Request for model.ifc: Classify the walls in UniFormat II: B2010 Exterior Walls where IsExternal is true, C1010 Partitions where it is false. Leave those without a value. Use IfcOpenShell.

First a look at what the model holds.

```python
import ifcopenshell
import ifcopenshell.util.element

model = ifcopenshell.open("model.ifc")
print(model.schema)
print("classifications:", [c.Name for c in model.by_type("IfcClassification")])
values = [ifcopenshell.util.element.get_pset(e, "Pset_WallCommon", "IsExternal") for e in model.by_type("IfcWall")]
for value in (True, False, None):
    print("IsExternal", value, values.count(value))
```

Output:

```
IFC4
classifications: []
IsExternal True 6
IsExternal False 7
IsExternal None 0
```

```python
import ifcopenshell
import ifcopenshell.api.classification
import ifcopenshell.util.element

model = ifcopenshell.open("model.ifc")

system = ifcopenshell.api.classification.add_classification(model, classification="UniFormat II")

walls = model.by_type("IfcWall")
external = {e: ifcopenshell.util.element.get_pset(e, "Pset_WallCommon", "IsExternal") for e in walls}
for flag, code, name in ((True, "B2010", "Exterior Walls"), (False, "C1010", "Partitions")):
    products = [e for e in walls if external[e] is flag]
    ifcopenshell.api.classification.add_reference(
        model, products=products, classification=system, identification=code, name=name
    )
    print(code, len(products))

model.write("model_edited.ifc")
```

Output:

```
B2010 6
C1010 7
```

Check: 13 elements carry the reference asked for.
